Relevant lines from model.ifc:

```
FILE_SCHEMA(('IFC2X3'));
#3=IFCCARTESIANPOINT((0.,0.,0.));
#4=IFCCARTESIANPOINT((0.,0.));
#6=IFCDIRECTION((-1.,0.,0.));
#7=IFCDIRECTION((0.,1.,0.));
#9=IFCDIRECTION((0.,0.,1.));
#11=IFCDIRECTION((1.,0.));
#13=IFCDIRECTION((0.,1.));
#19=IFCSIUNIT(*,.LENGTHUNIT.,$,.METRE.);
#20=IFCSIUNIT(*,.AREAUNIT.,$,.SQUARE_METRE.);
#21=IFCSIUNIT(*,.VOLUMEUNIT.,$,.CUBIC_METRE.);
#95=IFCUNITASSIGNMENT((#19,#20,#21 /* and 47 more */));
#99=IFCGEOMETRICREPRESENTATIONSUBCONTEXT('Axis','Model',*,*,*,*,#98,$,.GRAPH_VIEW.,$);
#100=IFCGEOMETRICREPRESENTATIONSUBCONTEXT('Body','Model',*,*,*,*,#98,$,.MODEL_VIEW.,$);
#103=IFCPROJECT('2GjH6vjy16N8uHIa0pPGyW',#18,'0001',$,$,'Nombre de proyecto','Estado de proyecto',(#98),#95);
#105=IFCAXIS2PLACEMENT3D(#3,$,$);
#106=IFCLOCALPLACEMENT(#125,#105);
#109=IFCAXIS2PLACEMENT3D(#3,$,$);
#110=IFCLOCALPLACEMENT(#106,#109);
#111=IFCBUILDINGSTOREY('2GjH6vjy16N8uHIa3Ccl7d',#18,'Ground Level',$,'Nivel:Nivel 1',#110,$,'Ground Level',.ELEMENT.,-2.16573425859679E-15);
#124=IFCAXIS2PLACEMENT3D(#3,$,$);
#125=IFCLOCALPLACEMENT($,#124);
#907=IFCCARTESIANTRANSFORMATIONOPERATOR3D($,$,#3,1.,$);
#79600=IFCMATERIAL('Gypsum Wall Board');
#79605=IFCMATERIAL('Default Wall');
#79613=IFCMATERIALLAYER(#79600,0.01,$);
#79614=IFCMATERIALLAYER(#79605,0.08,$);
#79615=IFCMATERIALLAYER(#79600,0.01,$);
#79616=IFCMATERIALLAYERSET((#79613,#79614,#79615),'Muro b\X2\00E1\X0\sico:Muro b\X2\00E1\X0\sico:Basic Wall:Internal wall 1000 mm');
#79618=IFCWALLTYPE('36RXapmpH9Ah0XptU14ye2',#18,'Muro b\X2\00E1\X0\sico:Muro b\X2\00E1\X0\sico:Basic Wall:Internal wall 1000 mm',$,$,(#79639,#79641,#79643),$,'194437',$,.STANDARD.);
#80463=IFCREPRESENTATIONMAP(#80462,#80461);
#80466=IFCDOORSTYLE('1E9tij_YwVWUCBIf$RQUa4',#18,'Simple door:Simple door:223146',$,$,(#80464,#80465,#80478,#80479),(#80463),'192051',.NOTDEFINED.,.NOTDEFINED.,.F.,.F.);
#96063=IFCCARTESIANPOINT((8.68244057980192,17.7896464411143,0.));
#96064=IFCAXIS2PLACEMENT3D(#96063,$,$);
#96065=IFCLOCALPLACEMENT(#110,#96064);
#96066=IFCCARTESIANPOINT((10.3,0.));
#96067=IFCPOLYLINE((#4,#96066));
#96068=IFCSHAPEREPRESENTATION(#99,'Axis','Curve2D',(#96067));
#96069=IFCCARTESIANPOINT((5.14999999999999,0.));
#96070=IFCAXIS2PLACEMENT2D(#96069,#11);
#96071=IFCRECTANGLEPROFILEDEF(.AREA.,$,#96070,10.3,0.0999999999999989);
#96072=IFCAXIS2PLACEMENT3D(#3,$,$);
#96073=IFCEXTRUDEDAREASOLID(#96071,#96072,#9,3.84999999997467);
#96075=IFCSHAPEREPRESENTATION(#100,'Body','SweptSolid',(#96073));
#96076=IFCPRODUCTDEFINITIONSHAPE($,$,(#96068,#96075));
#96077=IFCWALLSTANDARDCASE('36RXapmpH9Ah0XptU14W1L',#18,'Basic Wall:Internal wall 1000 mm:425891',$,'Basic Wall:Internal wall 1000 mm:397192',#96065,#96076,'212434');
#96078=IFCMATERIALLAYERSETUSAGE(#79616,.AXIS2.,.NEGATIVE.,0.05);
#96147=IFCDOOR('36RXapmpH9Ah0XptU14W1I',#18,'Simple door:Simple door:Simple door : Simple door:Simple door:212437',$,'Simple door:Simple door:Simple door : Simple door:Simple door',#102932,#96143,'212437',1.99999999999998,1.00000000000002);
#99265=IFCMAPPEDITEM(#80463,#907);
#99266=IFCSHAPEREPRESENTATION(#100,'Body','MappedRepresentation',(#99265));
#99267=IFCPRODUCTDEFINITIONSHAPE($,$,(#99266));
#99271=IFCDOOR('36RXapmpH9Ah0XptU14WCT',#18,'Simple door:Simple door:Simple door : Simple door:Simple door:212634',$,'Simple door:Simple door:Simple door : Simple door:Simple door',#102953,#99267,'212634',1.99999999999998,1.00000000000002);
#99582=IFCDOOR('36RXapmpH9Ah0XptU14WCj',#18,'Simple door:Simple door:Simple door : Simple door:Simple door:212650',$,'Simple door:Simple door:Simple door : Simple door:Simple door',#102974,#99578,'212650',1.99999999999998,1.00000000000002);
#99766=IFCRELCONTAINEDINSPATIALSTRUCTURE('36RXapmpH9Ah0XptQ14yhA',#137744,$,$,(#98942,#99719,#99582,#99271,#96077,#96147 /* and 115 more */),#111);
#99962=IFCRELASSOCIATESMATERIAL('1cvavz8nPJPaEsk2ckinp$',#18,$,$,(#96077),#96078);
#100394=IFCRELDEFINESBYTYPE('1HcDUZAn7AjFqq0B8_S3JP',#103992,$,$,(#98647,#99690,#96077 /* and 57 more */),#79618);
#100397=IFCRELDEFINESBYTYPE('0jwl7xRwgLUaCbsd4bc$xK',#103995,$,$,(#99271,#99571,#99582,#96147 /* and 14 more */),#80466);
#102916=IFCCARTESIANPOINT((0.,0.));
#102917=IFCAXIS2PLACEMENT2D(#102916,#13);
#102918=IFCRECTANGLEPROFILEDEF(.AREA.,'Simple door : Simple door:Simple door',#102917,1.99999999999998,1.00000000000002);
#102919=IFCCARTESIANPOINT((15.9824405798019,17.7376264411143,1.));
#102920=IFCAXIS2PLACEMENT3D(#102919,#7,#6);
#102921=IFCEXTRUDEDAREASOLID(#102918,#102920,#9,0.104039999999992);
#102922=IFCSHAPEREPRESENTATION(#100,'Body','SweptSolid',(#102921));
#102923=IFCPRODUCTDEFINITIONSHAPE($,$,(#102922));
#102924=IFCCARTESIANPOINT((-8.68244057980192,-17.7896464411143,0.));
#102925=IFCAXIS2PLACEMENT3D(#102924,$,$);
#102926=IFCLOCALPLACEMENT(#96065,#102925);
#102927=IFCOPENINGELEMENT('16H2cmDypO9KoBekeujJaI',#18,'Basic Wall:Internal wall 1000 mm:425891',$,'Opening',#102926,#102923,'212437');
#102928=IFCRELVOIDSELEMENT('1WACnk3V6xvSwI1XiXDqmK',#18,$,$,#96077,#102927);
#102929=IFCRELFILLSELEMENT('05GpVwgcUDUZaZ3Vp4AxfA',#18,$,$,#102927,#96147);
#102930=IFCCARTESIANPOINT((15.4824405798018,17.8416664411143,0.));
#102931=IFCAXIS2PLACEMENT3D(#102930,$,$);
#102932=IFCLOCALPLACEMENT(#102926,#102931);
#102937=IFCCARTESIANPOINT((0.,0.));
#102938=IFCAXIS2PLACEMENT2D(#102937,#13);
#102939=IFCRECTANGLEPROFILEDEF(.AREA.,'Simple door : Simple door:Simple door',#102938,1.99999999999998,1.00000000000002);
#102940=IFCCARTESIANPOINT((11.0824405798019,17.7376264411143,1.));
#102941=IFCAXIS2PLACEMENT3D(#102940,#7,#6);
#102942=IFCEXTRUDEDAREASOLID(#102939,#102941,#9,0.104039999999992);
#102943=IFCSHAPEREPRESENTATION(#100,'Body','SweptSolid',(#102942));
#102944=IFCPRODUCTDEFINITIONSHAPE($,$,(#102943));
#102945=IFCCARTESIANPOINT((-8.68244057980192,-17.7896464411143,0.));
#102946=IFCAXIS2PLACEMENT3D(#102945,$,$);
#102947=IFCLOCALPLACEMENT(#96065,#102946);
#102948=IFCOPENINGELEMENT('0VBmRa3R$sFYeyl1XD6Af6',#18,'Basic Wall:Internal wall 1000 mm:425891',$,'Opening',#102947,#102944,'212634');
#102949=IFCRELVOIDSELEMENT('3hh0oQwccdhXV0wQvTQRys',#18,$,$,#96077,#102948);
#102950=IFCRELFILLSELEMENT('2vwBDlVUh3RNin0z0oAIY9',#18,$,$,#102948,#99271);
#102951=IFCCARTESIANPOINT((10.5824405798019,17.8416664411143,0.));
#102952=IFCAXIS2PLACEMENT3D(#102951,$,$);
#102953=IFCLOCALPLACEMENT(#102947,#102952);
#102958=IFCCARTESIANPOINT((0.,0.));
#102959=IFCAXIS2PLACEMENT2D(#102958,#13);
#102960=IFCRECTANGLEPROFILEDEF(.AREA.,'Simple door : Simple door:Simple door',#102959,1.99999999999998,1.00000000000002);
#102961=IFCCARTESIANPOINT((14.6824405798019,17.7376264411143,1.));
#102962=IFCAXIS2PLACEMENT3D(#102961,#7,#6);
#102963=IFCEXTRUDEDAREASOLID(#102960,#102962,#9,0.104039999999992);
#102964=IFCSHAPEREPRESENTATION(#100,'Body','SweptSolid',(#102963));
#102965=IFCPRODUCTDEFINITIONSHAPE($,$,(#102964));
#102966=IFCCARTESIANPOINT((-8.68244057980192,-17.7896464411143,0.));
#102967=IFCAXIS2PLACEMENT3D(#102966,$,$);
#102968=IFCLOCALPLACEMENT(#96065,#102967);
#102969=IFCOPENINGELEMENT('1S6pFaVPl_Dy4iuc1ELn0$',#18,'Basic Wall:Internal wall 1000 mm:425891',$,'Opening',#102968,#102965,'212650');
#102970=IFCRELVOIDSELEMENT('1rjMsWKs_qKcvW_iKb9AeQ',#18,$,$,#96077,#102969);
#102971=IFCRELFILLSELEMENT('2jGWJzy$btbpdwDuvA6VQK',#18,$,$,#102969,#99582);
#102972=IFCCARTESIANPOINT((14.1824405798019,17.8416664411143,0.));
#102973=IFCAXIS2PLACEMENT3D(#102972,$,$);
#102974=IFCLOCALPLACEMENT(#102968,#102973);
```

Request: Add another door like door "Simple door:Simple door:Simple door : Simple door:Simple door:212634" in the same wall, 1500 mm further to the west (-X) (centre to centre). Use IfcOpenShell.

```python
import ifcopenshell
import ifcopenshell.api.feature
import ifcopenshell.api.geometry
import ifcopenshell.api.root
import ifcopenshell.geom
import ifcopenshell.util.element
import ifcopenshell.util.placement
import ifcopenshell.util.shape

model = ifcopenshell.open("model.ifc")
settings = ifcopenshell.geom.settings()


def volume(element):
    """Net volume in cubic metres, openings subtracted."""
    shape = ifcopenshell.geom.create_shape(settings, element)
    return ifcopenshell.util.shape.get_volume(shape.geometry)


def reuse_history(source, copy):
    """copy_class also copies each property set's owner history, people and application; keep the originals."""
    for rel in copy.IsDefinedBy:
        if rel.is_a("IfcRelDefinesByProperties") and (history := rel.RelatingPropertyDefinition.OwnerHistory):
            rel.RelatingPropertyDefinition.OwnerHistory = source.OwnerHistory
            ifcopenshell.util.element.remove_deep2(model, history)


door = model.by_guid("36RXapmpH9Ah0XptU14WCT")
opening = door.FillsVoids[0].RelatingOpeningElement
wall = opening.VoidsElements[0].RelatingBuildingElement
before = volume(wall)
shift = ifcopenshell.util.placement.get_local_placement(wall.ObjectPlacement)[:3, 0] * -1.5

# copy_class copies the void relationship, type, container and properties, but no geometry.
new_opening = ifcopenshell.api.root.copy_class(model, product=opening)
new_opening.Representation = ifcopenshell.util.element.copy_deep(
    model, opening.Representation, exclude=["IfcGeometricRepresentationContext", "IfcRepresentationMap"]
)
new_opening.Name = "Basic Wall:Internal wall 1000 mm"
new_opening.Tag = None
new_door = ifcopenshell.api.root.copy_class(model, product=door)
new_door.Representation = ifcopenshell.util.element.copy_deep(
    model, door.Representation, exclude=["IfcGeometricRepresentationContext", "IfcRepresentationMap"]
)
new_door.Name = "Simple door:Simple door:Simple door : Simple door:Simple door"
new_door.Tag = None
reuse_history(door, new_door)
fills = ifcopenshell.api.feature.add_filling(model, opening=new_opening, element=new_door)
fills.OwnerHistory = new_door.OwnerHistory  # required in IFC2X3

for old, new in ((opening, new_opening), (door, new_door)):
    matrix = ifcopenshell.util.placement.get_local_placement(old.ObjectPlacement)
    matrix[:3, 3] += shift
    ifcopenshell.api.geometry.edit_object_placement(model, product=new, matrix=matrix, is_si=False)

after = volume(wall)

print(f"wall volume {before:.3f} -> {after:.3f} m3")

model.write("model_edited.ifc")
```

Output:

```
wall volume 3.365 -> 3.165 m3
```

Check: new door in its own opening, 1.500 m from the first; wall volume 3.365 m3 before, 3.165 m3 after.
